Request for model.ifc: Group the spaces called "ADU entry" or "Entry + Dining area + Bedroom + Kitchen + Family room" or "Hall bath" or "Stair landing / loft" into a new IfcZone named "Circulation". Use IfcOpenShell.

First a look at what the model holds.

```python
import ifcopenshell

model = ifcopenshell.open("model.ifc")
print(model.schema)
seen = {}
for space in model.by_type("IfcSpace"):
    seen[space.Name] = seen.get(space.Name, 0) + 1
for name, count in sorted(seen.items(), key=str):
    print(count, "x", name)
print("zones:", [z.Name for z in model.by_type("IfcZone")][:20])
```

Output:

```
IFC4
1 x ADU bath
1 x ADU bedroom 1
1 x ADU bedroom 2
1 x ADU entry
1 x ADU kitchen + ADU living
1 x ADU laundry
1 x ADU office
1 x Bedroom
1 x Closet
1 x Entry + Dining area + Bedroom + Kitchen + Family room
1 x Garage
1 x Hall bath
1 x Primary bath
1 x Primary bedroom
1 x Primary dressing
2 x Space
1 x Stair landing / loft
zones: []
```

```python
import ifcopenshell
import ifcopenshell.api.group
import ifcopenshell.api.root

model = ifcopenshell.open("model.ifc")

names = {"ADU entry", "Entry + Dining area + Bedroom + Kitchen + Family room", "Hall bath", "Stair landing / loft"}
spaces = [s for s in model.by_type("IfcSpace") if s.Name in names]

zone = ifcopenshell.api.root.create_entity(model, ifc_class="IfcZone", name="Circulation")
ifcopenshell.api.group.assign_group(model, products=spaces, group=zone)
print(len(spaces), "spaces in", zone.Name)

model.write("model-out.ifc")
```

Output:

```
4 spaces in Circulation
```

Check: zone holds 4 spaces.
